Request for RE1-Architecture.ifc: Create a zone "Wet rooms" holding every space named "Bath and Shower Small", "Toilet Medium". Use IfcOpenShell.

First a look at what the model holds.

```python
import ifcopenshell

model = ifcopenshell.open("RE1-Architecture.ifc")
print(model.schema)
seen = {}
for space in model.by_type("IfcSpace"):
    seen[space.LongName] = seen.get(space.LongName, 0) + 1
for name, count in sorted(seen.items(), key=str):
    print(count, "x", name)
print("zones:", [z.Name for z in model.by_type("IfcZone")][:20])
```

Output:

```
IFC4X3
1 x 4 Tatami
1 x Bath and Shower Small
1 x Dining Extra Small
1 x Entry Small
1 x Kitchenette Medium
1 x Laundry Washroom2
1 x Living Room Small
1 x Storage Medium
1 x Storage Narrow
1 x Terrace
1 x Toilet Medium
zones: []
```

```python
import ifcopenshell
import ifcopenshell.api.group
import ifcopenshell.api.root

model = ifcopenshell.open("RE1-Architecture.ifc")

names = {"Bath and Shower Small", "Toilet Medium"}
spaces = [s for s in model.by_type("IfcSpace") if s.LongName in names]

zone = ifcopenshell.api.root.create_entity(model, ifc_class="IfcZone", name="Wet rooms")
ifcopenshell.api.group.assign_group(model, products=spaces, group=zone)
print(len(spaces), "spaces in", zone.Name)

model.write("RE1-Architecture_edited.ifc")
```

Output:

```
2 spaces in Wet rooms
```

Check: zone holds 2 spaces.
